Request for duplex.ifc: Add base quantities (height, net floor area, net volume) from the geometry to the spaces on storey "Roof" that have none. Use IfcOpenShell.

First a look at what the model holds.

```python
import ifcopenshell
import ifcopenshell.util.element
import ifcopenshell.util.unit

model = ifcopenshell.open("duplex.ifc")
print(model.schema)
for unit_type in ("LENGTHUNIT", "AREAUNIT", "VOLUMEUNIT"):
    print(unit_type, ifcopenshell.util.unit.calculate_unit_scale(model, unit_type))
storey = next(s for s in model.by_type("IfcBuildingStorey") if s.Name == "Roof")
spaces = [e for e in ifcopenshell.util.element.get_decomposition(storey) if e.is_a("IfcSpace")]
for e in sorted(spaces, key=lambda e: e.id()):
    print(e.id(), e.is_a(), e.Name, list(ifcopenshell.util.element.get_psets(e, qtos_only=True)), sep=" | ")
```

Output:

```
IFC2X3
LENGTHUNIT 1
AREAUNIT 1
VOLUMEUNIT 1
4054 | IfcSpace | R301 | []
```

```python
import ifcopenshell
import ifcopenshell.api.pset
import ifcopenshell.geom
import ifcopenshell.util.element
import ifcopenshell.util.shape
import ifcopenshell.util.unit

model = ifcopenshell.open("duplex.ifc")
unit_scale = ifcopenshell.util.unit.calculate_unit_scale(model)
area_scale = ifcopenshell.util.unit.calculate_unit_scale(model, "AREAUNIT")
volume_scale = ifcopenshell.util.unit.calculate_unit_scale(model, "VOLUMEUNIT")
settings = ifcopenshell.geom.settings()

storey = next(s for s in model.by_type("IfcBuildingStorey") if s.Name == "Roof")
spaces = [e for e in ifcopenshell.util.element.get_decomposition(storey) if e.is_a("IfcSpace")]

for e in sorted(spaces, key=lambda e: e.id()):
    if ifcopenshell.util.element.get_psets(e, qtos_only=True, should_inherit=False):
        continue
    # Geometry comes back in metres, in the element's own axes.
    shape = ifcopenshell.geom.create_shape(settings, e)
    values = {
        "Height": ifcopenshell.util.shape.get_z(shape.geometry) / unit_scale,
        "NetFloorArea": ifcopenshell.util.shape.get_footprint_area(shape.geometry) / area_scale,
        "NetVolume": ifcopenshell.util.shape.get_volume(shape.geometry) / volume_scale,
    }
    qto = ifcopenshell.api.pset.add_qto(model, product=e, name="BaseQuantities")
    ifcopenshell.api.pset.edit_qto(model, qto=qto, properties=values)
    print(e.id(), {k: round(v, 3) for k, v in values.items()})

model.write("duplex-out.ifc")
```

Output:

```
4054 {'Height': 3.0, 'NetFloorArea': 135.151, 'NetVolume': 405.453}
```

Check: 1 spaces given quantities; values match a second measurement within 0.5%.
